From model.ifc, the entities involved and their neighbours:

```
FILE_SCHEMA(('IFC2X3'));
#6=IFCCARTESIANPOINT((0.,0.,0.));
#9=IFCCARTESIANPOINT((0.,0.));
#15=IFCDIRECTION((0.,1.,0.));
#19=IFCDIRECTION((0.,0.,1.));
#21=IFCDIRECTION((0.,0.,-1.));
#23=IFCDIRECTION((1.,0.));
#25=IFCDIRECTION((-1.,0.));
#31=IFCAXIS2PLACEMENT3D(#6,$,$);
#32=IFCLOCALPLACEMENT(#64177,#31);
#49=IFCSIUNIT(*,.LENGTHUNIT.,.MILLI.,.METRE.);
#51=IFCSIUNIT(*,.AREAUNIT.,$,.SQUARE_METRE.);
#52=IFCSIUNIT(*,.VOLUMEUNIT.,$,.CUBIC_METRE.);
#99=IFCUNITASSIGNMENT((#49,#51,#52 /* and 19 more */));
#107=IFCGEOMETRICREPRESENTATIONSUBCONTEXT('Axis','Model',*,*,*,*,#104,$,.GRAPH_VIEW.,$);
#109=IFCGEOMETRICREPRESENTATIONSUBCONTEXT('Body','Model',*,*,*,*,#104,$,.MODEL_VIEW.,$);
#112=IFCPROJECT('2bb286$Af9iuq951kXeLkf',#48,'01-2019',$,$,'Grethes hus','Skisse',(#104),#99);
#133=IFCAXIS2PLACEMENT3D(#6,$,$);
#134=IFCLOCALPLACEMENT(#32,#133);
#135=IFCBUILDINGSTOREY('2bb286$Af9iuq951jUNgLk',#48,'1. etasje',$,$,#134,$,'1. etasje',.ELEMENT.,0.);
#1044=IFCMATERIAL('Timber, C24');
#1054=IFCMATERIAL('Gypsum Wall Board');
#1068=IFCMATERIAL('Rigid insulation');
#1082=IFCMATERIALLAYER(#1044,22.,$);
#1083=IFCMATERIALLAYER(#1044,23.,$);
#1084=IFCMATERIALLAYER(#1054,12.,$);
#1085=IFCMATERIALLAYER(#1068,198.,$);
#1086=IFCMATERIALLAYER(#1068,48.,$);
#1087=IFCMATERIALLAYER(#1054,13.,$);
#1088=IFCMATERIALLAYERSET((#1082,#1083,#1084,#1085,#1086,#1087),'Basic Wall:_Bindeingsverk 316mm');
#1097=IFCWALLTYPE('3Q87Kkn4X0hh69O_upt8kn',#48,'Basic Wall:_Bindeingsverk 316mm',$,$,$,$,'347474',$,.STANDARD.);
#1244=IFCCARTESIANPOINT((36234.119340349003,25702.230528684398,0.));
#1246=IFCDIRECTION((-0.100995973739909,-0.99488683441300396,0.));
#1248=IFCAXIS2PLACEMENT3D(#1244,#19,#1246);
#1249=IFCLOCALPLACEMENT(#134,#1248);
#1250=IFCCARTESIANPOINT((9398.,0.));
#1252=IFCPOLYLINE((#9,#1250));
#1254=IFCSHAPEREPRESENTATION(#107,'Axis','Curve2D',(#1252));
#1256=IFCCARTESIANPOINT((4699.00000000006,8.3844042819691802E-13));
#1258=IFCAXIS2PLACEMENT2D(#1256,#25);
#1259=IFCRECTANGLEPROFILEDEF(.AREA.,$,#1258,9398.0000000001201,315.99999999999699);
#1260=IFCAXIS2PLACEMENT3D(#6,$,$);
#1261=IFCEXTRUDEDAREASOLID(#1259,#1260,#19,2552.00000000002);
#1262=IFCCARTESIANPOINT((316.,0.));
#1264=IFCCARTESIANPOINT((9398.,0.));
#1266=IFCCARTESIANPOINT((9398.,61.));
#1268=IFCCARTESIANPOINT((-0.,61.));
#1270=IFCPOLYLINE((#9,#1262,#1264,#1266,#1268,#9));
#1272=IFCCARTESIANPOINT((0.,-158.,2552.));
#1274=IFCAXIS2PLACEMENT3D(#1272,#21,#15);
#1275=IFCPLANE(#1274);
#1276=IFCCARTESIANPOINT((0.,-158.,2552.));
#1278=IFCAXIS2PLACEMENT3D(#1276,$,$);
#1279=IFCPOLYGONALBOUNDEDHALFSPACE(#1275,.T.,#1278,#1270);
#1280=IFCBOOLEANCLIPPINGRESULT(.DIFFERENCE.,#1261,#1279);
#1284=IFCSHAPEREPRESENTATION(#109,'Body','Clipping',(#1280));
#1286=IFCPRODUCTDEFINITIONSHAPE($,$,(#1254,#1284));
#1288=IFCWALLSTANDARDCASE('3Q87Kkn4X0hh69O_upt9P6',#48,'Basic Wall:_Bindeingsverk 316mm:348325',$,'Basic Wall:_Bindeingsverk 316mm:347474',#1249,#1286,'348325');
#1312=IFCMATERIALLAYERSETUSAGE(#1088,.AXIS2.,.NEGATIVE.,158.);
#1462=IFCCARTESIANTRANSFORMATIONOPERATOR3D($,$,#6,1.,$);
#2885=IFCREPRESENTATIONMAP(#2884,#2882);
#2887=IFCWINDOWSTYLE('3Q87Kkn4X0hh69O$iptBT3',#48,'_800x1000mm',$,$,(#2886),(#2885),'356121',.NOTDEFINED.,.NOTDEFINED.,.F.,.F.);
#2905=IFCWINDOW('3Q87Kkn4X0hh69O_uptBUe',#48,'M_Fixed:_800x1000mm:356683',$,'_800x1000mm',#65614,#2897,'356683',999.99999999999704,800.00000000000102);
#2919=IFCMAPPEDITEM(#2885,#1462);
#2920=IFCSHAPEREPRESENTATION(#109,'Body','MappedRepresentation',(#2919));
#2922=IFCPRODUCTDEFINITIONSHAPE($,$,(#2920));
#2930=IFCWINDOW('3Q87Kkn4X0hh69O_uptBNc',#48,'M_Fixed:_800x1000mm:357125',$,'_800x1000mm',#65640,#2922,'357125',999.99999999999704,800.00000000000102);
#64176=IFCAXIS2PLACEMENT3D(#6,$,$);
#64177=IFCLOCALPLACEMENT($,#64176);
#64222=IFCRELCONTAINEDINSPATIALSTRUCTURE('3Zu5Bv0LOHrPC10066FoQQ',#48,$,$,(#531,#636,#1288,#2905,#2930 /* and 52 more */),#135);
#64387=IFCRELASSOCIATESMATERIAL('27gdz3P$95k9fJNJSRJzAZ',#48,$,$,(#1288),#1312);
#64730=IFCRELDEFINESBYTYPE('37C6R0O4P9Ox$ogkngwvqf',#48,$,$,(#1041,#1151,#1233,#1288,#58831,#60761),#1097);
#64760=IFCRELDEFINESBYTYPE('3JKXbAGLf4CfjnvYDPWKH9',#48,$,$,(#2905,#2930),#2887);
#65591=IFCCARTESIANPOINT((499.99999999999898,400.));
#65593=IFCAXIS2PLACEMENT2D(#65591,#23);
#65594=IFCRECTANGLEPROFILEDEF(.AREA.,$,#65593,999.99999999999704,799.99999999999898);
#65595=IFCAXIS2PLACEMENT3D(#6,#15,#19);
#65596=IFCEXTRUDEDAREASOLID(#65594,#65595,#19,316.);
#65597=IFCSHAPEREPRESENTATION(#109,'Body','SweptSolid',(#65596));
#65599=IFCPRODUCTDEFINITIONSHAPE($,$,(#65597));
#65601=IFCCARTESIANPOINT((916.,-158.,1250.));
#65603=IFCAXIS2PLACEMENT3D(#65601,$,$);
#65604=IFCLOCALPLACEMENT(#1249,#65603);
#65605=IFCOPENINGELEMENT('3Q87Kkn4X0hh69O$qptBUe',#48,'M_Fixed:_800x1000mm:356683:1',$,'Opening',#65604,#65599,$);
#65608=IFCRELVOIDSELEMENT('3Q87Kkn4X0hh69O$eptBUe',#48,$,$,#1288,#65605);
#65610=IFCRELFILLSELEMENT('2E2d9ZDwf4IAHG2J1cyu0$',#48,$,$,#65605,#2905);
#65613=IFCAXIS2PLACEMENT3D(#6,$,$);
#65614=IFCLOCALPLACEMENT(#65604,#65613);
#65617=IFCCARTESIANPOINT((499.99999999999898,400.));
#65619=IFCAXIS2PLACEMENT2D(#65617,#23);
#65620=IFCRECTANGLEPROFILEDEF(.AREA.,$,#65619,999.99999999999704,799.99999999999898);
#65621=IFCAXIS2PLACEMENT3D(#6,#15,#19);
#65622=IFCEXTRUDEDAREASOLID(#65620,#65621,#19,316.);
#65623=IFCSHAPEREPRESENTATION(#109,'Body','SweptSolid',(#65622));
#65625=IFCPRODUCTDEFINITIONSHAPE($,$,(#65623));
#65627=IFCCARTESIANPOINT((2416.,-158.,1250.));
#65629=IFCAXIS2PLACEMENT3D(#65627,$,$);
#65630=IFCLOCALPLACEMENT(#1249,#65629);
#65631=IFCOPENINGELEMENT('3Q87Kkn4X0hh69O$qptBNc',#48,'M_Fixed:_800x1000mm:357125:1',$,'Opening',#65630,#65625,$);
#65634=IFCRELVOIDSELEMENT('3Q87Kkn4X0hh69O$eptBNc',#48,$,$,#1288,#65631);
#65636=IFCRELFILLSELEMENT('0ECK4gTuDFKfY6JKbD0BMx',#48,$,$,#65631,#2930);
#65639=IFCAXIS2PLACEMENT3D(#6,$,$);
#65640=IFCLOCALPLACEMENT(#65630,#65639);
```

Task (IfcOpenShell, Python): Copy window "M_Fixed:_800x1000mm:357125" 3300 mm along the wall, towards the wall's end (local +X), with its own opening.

```python
import ifcopenshell
import ifcopenshell.api.feature
import ifcopenshell.api.geometry
import ifcopenshell.api.root
import ifcopenshell.geom
import ifcopenshell.util.element
import ifcopenshell.util.placement
import ifcopenshell.util.shape

model = ifcopenshell.open("model.ifc")
settings = ifcopenshell.geom.settings()


def volume(element):
    """Net volume in cubic metres, openings subtracted."""
    shape = ifcopenshell.geom.create_shape(settings, element)
    return ifcopenshell.util.shape.get_volume(shape.geometry)


def reuse_history(source, copy):
    """copy_class also copies each property set's owner history, people and application; keep the originals."""
    for rel in copy.IsDefinedBy:
        if rel.is_a("IfcRelDefinesByProperties") and (history := rel.RelatingPropertyDefinition.OwnerHistory):
            rel.RelatingPropertyDefinition.OwnerHistory = source.OwnerHistory
            ifcopenshell.util.element.remove_deep2(model, history)


window = model.by_guid("3Q87Kkn4X0hh69O_uptBNc")
opening = window.FillsVoids[0].RelatingOpeningElement
wall = opening.VoidsElements[0].RelatingBuildingElement
before = volume(wall)
shift = ifcopenshell.util.placement.get_local_placement(wall.ObjectPlacement)[:3, 0] * 3300.0

# copy_class copies the void relationship, type, container and properties, but no geometry.
new_opening = ifcopenshell.api.root.copy_class(model, product=opening)
new_opening.Representation = ifcopenshell.util.element.copy_deep(
    model, opening.Representation, exclude=["IfcGeometricRepresentationContext", "IfcRepresentationMap"]
)
new_opening.Name = "M_Fixed:_800x1000mm"
new_window = ifcopenshell.api.root.copy_class(model, product=window)
new_window.Representation = ifcopenshell.util.element.copy_deep(
    model, window.Representation, exclude=["IfcGeometricRepresentationContext", "IfcRepresentationMap"]
)
new_window.Name = "M_Fixed:_800x1000mm"
new_window.Tag = None
reuse_history(window, new_window)
fills = ifcopenshell.api.feature.add_filling(model, opening=new_opening, element=new_window)
fills.OwnerHistory = new_window.OwnerHistory  # required in IFC2X3

for old, new in ((opening, new_opening), (window, new_window)):
    matrix = ifcopenshell.util.placement.get_local_placement(old.ObjectPlacement)
    matrix[:3, 3] += shift
    ifcopenshell.api.geometry.edit_object_placement(model, product=new, matrix=matrix, is_si=False)

after = volume(wall)

print(f"wall volume {before:.3f} -> {after:.3f} m3")

model.write("model_rev.ifc")
```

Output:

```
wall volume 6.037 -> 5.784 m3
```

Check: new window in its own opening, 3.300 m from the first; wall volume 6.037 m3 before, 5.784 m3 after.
